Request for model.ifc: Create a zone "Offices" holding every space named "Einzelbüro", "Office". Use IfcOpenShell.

First a look at what the model holds.

```python
import ifcopenshell

model = ifcopenshell.open("model.ifc")
print(model.schema)
seen = {}
for space in model.by_type("IfcSpace"):
    seen[space.LongName] = seen.get(space.LongName, 0) + 1
for name, count in sorted(seen.items(), key=str):
    print(count, "x", name)
print("zones:", [z.Name for z in model.by_type("IfcZone")][:20])
```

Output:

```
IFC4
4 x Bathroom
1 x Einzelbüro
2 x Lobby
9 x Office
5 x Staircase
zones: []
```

```python
import ifcopenshell
import ifcopenshell.api.group
import ifcopenshell.api.root

model = ifcopenshell.open("model.ifc")

names = {"Einzelbüro", "Office"}
spaces = [s for s in model.by_type("IfcSpace") if s.LongName in names]

zone = ifcopenshell.api.root.create_entity(model, ifc_class="IfcZone", name="Offices")
ifcopenshell.api.group.assign_group(model, products=spaces, group=zone)
print(len(spaces), "spaces in", zone.Name)

model.write("model_updated.ifc")
```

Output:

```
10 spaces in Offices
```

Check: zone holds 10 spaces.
